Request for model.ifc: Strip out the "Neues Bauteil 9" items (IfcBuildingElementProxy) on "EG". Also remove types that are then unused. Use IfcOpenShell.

First a look at what the model holds.

```python
import ifcopenshell
import ifcopenshell.util.element

model = ifcopenshell.open("model.ifc")
print(model.schema)
storey = next(s for s in model.by_type("IfcBuildingStorey") if s.Name == "EG")
proxies = [e for e in ifcopenshell.util.element.get_decomposition(storey) if e.is_a("IfcBuildingElementProxy")]
seen = {}
for e in proxies:
    element_type = ifcopenshell.util.element.get_type(e)
    name = element_type.Name if element_type not in (None, e) else None
    seen[name] = seen.get(name, 0) + 1
for name, count in sorted(seen.items(), key=str):
    print(count, "x", name)
```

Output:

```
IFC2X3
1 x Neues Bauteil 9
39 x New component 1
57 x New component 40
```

```python
import ifcopenshell
import ifcopenshell.api.root
import ifcopenshell.util.element

model = ifcopenshell.open("model.ifc")

storey = next(s for s in model.by_type("IfcBuildingStorey") if s.Name == "EG")
proxies = [e for e in ifcopenshell.util.element.get_decomposition(storey) if e.is_a("IfcBuildingElementProxy")]
targets = [e for e in proxies if (t := ifcopenshell.util.element.get_type(e)) not in (None, e) and t.Name == "Neues Bauteil 9"]
types = {ifcopenshell.util.element.get_type(e) for e in targets} - {None, *targets}

for e in targets:
    ifcopenshell.api.root.remove_product(model, product=e)
print(len(targets), "removed")

unused = [t for t in types if not ifcopenshell.util.element.get_types(t)]
for t in unused:
    ifcopenshell.api.root.remove_product(model, product=t)
print(len(unused), "unused types removed")

model.write("model_v2.ifc")
```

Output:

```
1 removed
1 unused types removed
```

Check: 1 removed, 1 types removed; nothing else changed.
